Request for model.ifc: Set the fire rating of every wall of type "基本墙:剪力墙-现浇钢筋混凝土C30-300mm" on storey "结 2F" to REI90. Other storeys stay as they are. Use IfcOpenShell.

First a look at what the model holds.

```python
import ifcopenshell
import ifcopenshell.util.element

model = ifcopenshell.open("model.ifc")
print(model.schema)
storey = next(s for s in model.by_type("IfcBuildingStorey") if s.Name == "结 2F")
walls = [e for e in ifcopenshell.util.element.get_decomposition(storey) if e.is_a("IfcWall")]
seen = {}
for e in walls:
    element_type = ifcopenshell.util.element.get_type(e)
    key = (element_type.Name if element_type != e and element_type else None, ifcopenshell.util.element.get_pset(e, "Pset_WallCommon", "FireRating"))
    seen[key] = seen.get(key, 0) + 1
for (name, value), count in sorted(seen.items(), key=str):
    print(count, "x", name, "|", value)
```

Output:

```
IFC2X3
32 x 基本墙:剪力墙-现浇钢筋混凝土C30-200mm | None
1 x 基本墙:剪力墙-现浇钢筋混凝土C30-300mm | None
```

```python
import ifcopenshell
import ifcopenshell.api.pset
import ifcopenshell.util.element

model = ifcopenshell.open("model.ifc")

storey = next(s for s in model.by_type("IfcBuildingStorey") if s.Name == "结 2F")
walls = [e for e in ifcopenshell.util.element.get_decomposition(storey) if e.is_a("IfcWall")]

count = 0
for e in walls:
    element_type = ifcopenshell.util.element.get_type(e)
    if element_type in (None, e) or element_type.Name != "基本墙:剪力墙-现浇钢筋混凝土C30-300mm":
        continue
    # add_pset returns the element's existing set when there is one.
    pset = ifcopenshell.api.pset.add_pset(model, product=e, name="Pset_WallCommon")
    ifcopenshell.api.pset.edit_pset(model, pset=pset, properties={"FireRating": "REI90"})
    count += 1

print(count, "walls updated")

model.write("model_edited.ifc")
```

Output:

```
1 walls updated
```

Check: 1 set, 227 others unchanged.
